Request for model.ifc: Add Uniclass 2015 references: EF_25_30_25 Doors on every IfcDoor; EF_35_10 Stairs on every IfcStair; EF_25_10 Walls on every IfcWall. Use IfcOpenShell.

First a look at what the model holds.

```python
import ifcopenshell

model = ifcopenshell.open("model.ifc")
print(model.schema)
print("classifications:", [c.Name for c in model.by_type("IfcClassification")])
for ifc_class in ("IfcDoor", "IfcRoof", "IfcStair", "IfcWall", "IfcWindow"):
    print(ifc_class, len(model.by_type(ifc_class)))
```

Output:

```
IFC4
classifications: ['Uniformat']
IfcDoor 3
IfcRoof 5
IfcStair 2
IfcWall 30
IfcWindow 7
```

```python
import ifcopenshell
import ifcopenshell.api.classification

model = ifcopenshell.open("model.ifc")

system = ifcopenshell.api.classification.add_classification(model, classification="Uniclass 2015")

codes = {
    "IfcDoor": ("EF_25_30_25", "Doors"),
    "IfcStair": ("EF_35_10", "Stairs"),
    "IfcWall": ("EF_25_10", "Walls"),
}
for ifc_class, (code, name) in codes.items():
    products = model.by_type(ifc_class)
    ifcopenshell.api.classification.add_reference(
        model, products=products, classification=system, identification=code, name=name
    )
    print(code, len(products))

model.write("model_rev.ifc")
```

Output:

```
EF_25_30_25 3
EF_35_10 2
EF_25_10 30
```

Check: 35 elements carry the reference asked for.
